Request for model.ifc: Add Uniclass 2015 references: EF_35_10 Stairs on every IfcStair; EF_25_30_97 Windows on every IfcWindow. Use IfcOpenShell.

First a look at what the model holds.

```python
import ifcopenshell

model = ifcopenshell.open("model.ifc")
print(model.schema)
print("classifications:", [c.Name for c in model.by_type("IfcClassification")])
for ifc_class in ("IfcDoor", "IfcRoof", "IfcStair", "IfcWall", "IfcWindow"):
    print(ifc_class, len(model.by_type(ifc_class)))
```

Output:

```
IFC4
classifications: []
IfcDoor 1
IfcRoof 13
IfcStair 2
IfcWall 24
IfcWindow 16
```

```python
import ifcopenshell
import ifcopenshell.api.classification

model = ifcopenshell.open("model.ifc")

system = ifcopenshell.api.classification.add_classification(model, classification="Uniclass 2015")

codes = {
    "IfcStair": ("EF_35_10", "Stairs"),
    "IfcWindow": ("EF_25_30_97", "Windows"),
}
for ifc_class, (code, name) in codes.items():
    products = model.by_type(ifc_class)
    ifcopenshell.api.classification.add_reference(
        model, products=products, classification=system, identification=code, name=name
    )
    print(code, len(products))

model.write("model_rev.ifc")
```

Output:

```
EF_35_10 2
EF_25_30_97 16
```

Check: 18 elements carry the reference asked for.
